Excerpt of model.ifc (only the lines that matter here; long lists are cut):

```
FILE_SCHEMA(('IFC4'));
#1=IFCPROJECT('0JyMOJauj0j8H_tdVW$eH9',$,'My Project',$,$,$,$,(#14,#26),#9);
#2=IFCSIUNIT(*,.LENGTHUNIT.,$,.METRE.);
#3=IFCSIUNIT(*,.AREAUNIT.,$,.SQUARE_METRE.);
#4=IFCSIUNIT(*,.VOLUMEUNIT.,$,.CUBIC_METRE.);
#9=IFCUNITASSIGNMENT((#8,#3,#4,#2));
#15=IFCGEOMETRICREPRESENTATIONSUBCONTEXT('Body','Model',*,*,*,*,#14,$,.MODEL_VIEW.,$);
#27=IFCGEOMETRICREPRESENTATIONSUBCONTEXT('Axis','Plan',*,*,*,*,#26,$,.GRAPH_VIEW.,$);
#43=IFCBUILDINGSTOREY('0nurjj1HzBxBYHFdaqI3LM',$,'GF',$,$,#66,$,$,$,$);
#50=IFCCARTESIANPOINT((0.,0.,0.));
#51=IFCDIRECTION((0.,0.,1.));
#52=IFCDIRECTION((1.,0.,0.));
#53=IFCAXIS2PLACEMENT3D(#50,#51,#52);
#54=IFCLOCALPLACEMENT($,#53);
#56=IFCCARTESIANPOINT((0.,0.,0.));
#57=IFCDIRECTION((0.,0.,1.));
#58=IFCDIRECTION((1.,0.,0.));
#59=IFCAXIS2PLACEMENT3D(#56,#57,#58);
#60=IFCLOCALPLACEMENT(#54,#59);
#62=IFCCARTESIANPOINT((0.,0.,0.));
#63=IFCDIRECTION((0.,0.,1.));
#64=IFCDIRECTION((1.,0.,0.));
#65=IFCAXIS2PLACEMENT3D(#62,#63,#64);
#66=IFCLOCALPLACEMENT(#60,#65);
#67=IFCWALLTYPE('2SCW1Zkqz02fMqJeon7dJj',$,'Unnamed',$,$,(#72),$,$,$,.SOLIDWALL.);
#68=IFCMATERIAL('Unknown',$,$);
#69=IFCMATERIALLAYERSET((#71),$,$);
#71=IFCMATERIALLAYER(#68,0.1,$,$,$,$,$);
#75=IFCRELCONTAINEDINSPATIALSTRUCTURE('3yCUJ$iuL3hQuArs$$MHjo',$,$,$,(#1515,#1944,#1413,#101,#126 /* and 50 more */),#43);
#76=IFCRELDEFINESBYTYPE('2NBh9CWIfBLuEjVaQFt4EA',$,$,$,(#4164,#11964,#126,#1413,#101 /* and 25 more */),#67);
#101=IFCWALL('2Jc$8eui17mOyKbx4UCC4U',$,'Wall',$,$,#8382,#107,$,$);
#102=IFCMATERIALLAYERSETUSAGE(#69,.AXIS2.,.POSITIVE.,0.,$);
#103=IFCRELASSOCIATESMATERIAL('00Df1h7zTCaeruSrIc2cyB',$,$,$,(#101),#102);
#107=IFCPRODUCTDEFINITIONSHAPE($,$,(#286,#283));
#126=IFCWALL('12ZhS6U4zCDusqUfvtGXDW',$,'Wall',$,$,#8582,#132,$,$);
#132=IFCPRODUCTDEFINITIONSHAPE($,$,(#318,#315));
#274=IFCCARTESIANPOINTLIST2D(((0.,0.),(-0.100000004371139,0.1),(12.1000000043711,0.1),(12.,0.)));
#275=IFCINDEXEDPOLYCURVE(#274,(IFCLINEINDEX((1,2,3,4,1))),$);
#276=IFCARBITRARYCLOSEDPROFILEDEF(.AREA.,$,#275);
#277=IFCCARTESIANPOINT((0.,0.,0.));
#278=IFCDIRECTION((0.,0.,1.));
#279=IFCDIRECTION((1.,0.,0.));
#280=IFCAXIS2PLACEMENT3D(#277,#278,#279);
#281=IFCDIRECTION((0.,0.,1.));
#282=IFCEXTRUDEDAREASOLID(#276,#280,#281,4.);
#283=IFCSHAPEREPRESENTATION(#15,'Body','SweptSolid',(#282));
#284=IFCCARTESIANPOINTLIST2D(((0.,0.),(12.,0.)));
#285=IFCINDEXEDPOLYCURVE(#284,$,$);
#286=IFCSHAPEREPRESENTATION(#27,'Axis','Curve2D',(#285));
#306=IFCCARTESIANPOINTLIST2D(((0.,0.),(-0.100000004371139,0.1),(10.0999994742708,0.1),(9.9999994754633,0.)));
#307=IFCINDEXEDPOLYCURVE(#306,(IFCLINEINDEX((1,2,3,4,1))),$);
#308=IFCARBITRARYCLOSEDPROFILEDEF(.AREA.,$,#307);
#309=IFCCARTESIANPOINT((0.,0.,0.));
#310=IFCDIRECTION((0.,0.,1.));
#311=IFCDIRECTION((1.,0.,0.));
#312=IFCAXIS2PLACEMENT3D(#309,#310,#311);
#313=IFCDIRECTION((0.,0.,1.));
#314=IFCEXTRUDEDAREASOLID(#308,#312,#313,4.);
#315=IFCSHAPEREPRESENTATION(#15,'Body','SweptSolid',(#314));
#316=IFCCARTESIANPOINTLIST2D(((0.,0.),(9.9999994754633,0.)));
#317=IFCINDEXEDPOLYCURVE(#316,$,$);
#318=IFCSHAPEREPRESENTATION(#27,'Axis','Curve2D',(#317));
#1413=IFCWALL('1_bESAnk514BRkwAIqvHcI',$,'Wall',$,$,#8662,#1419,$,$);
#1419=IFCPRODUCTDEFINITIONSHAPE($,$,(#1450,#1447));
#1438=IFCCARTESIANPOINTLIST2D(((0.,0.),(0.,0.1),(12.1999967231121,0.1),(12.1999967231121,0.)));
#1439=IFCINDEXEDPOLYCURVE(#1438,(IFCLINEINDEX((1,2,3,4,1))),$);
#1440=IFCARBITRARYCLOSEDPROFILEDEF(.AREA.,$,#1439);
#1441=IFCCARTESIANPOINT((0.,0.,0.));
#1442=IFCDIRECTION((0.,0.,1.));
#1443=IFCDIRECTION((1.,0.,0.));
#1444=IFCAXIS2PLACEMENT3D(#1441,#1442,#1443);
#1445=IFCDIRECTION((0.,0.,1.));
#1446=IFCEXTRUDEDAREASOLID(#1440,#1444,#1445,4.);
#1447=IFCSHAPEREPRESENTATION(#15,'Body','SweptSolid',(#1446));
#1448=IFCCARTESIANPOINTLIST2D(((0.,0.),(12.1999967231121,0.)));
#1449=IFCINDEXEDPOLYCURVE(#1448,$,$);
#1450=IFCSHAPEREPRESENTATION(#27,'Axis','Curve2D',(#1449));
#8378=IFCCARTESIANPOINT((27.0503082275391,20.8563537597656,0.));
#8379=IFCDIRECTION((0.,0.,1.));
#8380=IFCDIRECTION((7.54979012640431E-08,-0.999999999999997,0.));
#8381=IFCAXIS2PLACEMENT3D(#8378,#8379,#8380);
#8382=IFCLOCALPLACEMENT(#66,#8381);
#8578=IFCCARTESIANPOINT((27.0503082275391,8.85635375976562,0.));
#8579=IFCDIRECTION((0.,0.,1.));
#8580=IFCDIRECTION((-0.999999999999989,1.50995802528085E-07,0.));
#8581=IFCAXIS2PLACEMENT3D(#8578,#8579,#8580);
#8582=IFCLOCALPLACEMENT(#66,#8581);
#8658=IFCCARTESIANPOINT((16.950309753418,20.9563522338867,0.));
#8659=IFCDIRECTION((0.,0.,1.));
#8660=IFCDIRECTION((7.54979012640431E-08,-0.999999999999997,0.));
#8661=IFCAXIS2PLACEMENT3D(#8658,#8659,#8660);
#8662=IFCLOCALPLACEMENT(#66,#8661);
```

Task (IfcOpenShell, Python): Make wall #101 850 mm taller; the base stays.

```python
import ifcopenshell
import ifcopenshell.geom
import ifcopenshell.util.representation
import ifcopenshell.util.shape
import ifcopenshell.util.unit

model = ifcopenshell.open("model.ifc")
unit_scale = ifcopenshell.util.unit.calculate_unit_scale(model)
settings = ifcopenshell.geom.settings()


def volume(element):
    """Net volume in cubic metres, openings subtracted."""
    shape = ifcopenshell.geom.create_shape(settings, element)
    return ifcopenshell.util.shape.get_volume(shape.geometry)


wall = model.by_guid("2Jc$8eui17mOyKbx4UCC4U")
before = volume(wall)

body = ifcopenshell.util.representation.get_representation(wall, "Model", "Body")
solid = body.Items[0]
old_height = solid.Depth
solid.Depth += 0.85 / unit_scale
after = volume(wall)

print(f"height {old_height:g} -> {solid.Depth:g}, volume {before:.3f} -> {after:.3f} m3")

model.write("model_edited.ifc")
```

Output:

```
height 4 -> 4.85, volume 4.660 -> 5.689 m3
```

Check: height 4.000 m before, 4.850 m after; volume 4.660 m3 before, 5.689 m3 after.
